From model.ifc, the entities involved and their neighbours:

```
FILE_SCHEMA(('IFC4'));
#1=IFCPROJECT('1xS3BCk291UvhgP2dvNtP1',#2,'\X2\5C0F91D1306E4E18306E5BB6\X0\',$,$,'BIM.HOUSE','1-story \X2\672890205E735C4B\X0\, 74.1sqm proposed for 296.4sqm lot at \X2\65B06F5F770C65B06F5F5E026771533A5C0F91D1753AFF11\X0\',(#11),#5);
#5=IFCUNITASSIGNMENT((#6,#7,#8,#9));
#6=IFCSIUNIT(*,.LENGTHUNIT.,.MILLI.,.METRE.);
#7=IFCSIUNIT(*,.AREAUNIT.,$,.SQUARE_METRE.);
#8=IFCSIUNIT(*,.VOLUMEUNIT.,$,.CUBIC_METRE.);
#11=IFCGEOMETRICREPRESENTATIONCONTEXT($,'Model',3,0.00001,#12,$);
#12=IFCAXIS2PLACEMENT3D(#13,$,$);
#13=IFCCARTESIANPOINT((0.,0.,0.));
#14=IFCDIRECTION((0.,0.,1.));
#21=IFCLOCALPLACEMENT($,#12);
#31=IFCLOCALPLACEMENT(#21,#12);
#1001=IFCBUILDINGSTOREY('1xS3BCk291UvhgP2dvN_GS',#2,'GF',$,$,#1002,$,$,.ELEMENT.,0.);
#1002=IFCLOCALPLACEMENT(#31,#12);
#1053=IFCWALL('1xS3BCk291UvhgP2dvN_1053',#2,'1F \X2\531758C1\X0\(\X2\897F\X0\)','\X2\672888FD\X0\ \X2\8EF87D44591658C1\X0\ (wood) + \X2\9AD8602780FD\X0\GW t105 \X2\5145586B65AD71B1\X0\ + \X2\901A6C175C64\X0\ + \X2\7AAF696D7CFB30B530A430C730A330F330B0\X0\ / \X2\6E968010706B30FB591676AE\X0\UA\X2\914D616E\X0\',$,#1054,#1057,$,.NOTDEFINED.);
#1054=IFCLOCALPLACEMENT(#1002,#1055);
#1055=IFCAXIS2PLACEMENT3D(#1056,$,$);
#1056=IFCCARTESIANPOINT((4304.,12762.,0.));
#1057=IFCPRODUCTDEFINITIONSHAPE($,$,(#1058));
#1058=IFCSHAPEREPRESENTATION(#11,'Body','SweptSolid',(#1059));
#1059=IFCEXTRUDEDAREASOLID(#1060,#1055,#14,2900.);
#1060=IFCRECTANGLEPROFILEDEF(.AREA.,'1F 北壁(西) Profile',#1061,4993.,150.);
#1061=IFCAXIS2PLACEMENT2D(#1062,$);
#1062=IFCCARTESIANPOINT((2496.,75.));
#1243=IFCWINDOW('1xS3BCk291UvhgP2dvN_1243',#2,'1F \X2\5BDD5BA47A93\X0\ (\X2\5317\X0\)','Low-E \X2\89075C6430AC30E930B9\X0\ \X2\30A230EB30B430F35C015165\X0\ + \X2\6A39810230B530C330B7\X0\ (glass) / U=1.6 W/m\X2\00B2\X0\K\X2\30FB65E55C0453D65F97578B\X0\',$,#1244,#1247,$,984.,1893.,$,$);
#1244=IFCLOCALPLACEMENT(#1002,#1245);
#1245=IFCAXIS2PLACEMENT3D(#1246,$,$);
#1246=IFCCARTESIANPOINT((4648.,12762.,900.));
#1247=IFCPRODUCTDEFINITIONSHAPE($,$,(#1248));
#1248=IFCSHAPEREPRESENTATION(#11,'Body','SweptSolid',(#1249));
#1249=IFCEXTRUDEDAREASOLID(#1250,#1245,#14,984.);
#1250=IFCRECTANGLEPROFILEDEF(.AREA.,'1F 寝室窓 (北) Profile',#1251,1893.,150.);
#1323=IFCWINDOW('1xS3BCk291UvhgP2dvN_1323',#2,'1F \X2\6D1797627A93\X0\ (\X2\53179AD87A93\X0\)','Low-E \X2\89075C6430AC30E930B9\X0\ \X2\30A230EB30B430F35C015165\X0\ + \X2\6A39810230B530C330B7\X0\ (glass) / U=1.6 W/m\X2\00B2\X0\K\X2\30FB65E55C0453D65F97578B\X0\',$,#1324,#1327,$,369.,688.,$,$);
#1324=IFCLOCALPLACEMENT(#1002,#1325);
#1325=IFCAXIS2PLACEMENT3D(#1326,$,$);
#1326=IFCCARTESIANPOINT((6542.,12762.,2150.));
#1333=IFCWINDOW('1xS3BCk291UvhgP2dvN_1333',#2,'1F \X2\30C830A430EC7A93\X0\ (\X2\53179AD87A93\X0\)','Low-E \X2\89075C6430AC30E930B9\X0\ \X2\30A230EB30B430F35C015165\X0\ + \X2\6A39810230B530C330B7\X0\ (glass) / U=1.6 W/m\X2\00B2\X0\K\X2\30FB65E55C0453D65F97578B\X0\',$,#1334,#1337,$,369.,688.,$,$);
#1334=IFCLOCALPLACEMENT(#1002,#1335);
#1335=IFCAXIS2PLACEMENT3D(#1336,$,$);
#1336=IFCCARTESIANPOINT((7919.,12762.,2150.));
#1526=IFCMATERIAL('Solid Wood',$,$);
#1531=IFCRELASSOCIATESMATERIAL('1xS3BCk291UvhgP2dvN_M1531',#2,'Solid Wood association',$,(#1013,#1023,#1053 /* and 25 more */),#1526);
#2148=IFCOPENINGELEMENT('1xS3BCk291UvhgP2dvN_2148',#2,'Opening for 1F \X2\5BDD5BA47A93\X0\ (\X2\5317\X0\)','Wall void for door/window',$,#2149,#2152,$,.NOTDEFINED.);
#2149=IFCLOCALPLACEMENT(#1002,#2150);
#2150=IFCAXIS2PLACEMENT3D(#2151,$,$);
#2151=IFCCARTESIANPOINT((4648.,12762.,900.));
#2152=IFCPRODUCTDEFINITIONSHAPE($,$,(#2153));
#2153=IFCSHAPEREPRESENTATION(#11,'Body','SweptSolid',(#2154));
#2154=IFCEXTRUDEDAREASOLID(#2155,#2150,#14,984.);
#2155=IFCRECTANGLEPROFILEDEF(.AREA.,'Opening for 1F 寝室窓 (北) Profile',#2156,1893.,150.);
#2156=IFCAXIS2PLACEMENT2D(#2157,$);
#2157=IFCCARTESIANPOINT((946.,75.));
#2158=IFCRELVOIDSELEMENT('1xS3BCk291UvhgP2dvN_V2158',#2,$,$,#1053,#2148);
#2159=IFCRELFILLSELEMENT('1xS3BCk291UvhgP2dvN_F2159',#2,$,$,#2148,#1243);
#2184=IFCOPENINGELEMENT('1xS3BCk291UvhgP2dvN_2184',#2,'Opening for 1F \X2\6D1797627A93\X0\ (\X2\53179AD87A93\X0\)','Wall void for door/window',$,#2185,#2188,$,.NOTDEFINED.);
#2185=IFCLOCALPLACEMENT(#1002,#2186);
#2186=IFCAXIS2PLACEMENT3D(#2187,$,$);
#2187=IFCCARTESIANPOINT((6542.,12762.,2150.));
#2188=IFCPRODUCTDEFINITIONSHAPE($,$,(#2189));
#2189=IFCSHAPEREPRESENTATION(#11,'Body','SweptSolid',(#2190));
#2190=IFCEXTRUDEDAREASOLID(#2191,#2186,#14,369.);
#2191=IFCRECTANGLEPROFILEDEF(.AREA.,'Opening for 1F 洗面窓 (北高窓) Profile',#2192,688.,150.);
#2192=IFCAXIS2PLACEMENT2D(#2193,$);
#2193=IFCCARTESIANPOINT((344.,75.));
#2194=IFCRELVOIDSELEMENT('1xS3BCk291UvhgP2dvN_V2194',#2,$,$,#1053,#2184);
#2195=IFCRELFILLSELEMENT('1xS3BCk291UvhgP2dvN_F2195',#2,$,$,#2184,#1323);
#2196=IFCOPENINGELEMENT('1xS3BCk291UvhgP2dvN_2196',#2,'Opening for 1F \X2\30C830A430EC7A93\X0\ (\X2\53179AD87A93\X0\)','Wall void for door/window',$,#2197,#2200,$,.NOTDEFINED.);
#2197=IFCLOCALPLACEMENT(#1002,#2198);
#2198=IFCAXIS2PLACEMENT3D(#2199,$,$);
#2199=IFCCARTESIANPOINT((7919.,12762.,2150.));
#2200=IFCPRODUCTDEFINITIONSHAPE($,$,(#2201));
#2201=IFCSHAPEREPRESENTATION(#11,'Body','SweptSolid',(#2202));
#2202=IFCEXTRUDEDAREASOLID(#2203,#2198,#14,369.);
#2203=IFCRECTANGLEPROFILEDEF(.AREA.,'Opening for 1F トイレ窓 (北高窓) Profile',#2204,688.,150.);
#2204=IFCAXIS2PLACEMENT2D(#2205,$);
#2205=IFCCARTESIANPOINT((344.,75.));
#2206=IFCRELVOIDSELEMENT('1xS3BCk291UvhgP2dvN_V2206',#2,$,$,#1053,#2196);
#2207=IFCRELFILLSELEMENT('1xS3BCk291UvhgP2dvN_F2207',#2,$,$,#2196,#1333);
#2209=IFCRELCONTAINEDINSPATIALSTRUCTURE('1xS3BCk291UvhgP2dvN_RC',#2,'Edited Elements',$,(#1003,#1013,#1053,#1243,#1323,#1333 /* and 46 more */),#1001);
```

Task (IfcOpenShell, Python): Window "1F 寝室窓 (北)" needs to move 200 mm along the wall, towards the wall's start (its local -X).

```python
import ifcopenshell
import ifcopenshell.api.geometry
import ifcopenshell.util.placement
import ifcopenshell.util.unit

model = ifcopenshell.open("model.ifc")
unit_scale = ifcopenshell.util.unit.calculate_unit_scale(model)

window = model.by_guid("1xS3BCk291UvhgP2dvN_1243")
opening = window.FillsVoids[0].RelatingOpeningElement
wall = opening.VoidsElements[0].RelatingBuildingElement

wall_matrix = ifcopenshell.util.placement.get_local_placement(wall.ObjectPlacement)
shift = wall_matrix[:3, 0] * -0.2 / unit_scale
before = ifcopenshell.util.placement.get_local_placement(window.ObjectPlacement)[:3, 3].copy()

# The window is not placed relative to its opening, so move both.
for product in (opening, window):
    matrix = ifcopenshell.util.placement.get_local_placement(product.ObjectPlacement)
    matrix[:3, 3] += shift
    ifcopenshell.api.geometry.edit_object_placement(model, product=product, matrix=matrix, is_si=False)

after = ifcopenshell.util.placement.get_local_placement(window.ObjectPlacement)[:3, 3]
print("window moved by", (after - before).round(3) + 0.0)

model.write("model-out.ifc")
```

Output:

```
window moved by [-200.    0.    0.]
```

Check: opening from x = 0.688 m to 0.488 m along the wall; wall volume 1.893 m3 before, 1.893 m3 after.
